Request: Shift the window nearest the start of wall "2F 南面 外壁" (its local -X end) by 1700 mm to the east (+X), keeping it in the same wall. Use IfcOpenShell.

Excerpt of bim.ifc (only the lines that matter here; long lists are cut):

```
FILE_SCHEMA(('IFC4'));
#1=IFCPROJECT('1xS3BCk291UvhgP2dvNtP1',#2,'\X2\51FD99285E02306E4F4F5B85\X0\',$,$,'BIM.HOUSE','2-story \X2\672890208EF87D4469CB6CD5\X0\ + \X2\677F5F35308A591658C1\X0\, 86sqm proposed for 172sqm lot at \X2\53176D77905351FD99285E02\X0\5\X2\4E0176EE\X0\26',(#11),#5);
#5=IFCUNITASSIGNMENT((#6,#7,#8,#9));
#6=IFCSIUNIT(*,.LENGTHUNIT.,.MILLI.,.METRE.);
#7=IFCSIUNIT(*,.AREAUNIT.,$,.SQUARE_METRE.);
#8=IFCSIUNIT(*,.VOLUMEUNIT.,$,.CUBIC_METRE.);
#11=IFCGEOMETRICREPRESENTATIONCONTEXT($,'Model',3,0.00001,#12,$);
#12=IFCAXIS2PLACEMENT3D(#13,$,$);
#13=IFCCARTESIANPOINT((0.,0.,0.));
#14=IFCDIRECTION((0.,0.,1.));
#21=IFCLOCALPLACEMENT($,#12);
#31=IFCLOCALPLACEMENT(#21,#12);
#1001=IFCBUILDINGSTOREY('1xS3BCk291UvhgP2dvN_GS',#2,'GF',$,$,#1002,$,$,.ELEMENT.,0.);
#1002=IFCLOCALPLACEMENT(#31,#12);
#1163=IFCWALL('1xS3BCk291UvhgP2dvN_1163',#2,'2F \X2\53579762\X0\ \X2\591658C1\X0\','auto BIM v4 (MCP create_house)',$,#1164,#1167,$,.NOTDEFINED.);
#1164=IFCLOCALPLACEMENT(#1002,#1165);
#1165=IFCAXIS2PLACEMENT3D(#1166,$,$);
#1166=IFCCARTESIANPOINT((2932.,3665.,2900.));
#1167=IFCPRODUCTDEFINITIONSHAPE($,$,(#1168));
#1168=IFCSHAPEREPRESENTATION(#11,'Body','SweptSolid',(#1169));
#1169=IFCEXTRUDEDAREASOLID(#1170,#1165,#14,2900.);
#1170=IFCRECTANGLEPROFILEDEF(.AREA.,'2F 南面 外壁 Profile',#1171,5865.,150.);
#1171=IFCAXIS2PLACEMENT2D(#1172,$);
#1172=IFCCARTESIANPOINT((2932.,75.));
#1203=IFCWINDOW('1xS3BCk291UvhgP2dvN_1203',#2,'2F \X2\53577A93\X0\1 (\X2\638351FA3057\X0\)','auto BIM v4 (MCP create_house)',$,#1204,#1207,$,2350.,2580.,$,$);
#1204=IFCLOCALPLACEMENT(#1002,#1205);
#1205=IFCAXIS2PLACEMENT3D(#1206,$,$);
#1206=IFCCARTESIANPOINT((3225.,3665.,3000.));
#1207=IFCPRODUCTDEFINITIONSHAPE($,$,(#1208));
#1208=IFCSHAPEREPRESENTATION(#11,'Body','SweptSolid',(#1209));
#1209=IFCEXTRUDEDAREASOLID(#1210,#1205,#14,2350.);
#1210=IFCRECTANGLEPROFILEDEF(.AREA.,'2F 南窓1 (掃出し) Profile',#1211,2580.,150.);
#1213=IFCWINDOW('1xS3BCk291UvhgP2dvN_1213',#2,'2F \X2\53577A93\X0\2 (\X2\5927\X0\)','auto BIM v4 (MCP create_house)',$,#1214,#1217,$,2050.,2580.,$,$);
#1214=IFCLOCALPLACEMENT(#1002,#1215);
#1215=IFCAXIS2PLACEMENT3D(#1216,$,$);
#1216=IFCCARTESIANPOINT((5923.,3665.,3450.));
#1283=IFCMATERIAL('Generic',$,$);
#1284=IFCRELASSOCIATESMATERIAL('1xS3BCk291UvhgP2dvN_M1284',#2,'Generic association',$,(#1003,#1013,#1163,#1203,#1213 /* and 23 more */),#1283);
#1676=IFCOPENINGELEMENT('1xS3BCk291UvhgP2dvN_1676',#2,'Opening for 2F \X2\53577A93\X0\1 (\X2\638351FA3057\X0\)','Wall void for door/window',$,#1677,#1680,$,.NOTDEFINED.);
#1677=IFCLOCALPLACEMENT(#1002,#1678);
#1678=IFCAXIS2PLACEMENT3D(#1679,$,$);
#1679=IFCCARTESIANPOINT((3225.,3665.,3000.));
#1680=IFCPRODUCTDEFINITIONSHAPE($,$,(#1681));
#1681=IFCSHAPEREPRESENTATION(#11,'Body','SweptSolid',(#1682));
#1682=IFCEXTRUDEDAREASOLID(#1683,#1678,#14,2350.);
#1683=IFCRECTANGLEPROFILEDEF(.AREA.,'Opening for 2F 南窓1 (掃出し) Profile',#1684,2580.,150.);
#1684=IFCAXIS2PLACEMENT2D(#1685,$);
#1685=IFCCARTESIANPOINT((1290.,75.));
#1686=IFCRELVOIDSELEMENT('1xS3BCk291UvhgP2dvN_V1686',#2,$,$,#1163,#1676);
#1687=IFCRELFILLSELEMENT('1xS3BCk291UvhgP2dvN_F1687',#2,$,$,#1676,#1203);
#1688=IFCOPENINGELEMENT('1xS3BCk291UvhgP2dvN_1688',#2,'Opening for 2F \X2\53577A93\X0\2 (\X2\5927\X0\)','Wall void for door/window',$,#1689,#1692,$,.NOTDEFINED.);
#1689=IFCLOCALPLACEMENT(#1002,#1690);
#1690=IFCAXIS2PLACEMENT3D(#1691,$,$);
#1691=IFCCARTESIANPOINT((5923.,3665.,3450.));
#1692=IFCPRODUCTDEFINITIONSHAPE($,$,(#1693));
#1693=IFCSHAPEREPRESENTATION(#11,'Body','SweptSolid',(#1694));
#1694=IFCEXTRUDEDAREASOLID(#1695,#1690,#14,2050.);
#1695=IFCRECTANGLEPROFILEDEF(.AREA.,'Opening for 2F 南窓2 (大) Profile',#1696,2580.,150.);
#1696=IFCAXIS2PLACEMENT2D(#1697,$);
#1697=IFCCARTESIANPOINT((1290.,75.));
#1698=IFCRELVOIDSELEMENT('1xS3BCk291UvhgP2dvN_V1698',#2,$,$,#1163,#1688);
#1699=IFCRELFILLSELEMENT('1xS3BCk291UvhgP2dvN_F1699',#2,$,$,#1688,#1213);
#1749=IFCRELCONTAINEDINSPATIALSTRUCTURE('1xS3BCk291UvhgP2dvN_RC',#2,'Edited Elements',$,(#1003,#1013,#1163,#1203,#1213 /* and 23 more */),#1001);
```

```python
import ifcopenshell
import ifcopenshell.api.geometry
import ifcopenshell.util.placement
import ifcopenshell.util.unit

model = ifcopenshell.open("bim.ifc")
unit_scale = ifcopenshell.util.unit.calculate_unit_scale(model)

window = model.by_guid("1xS3BCk291UvhgP2dvN_1203")
opening = window.FillsVoids[0].RelatingOpeningElement
wall = opening.VoidsElements[0].RelatingBuildingElement

wall_matrix = ifcopenshell.util.placement.get_local_placement(wall.ObjectPlacement)
shift = wall_matrix[:3, 0] * 1.7 / unit_scale
before = ifcopenshell.util.placement.get_local_placement(window.ObjectPlacement)[:3, 3].copy()

# The window is not placed relative to its opening, so move both.
for product in (opening, window):
    matrix = ifcopenshell.util.placement.get_local_placement(product.ObjectPlacement)
    matrix[:3, 3] += shift
    ifcopenshell.api.geometry.edit_object_placement(model, product=product, matrix=matrix, is_si=False)

after = ifcopenshell.util.placement.get_local_placement(window.ObjectPlacement)[:3, 3]
print("window moved by", (after - before).round(3) + 0.0)

model.write("bim_edited.ifc")
```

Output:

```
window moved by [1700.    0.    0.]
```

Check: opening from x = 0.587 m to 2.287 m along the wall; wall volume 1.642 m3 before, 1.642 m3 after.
